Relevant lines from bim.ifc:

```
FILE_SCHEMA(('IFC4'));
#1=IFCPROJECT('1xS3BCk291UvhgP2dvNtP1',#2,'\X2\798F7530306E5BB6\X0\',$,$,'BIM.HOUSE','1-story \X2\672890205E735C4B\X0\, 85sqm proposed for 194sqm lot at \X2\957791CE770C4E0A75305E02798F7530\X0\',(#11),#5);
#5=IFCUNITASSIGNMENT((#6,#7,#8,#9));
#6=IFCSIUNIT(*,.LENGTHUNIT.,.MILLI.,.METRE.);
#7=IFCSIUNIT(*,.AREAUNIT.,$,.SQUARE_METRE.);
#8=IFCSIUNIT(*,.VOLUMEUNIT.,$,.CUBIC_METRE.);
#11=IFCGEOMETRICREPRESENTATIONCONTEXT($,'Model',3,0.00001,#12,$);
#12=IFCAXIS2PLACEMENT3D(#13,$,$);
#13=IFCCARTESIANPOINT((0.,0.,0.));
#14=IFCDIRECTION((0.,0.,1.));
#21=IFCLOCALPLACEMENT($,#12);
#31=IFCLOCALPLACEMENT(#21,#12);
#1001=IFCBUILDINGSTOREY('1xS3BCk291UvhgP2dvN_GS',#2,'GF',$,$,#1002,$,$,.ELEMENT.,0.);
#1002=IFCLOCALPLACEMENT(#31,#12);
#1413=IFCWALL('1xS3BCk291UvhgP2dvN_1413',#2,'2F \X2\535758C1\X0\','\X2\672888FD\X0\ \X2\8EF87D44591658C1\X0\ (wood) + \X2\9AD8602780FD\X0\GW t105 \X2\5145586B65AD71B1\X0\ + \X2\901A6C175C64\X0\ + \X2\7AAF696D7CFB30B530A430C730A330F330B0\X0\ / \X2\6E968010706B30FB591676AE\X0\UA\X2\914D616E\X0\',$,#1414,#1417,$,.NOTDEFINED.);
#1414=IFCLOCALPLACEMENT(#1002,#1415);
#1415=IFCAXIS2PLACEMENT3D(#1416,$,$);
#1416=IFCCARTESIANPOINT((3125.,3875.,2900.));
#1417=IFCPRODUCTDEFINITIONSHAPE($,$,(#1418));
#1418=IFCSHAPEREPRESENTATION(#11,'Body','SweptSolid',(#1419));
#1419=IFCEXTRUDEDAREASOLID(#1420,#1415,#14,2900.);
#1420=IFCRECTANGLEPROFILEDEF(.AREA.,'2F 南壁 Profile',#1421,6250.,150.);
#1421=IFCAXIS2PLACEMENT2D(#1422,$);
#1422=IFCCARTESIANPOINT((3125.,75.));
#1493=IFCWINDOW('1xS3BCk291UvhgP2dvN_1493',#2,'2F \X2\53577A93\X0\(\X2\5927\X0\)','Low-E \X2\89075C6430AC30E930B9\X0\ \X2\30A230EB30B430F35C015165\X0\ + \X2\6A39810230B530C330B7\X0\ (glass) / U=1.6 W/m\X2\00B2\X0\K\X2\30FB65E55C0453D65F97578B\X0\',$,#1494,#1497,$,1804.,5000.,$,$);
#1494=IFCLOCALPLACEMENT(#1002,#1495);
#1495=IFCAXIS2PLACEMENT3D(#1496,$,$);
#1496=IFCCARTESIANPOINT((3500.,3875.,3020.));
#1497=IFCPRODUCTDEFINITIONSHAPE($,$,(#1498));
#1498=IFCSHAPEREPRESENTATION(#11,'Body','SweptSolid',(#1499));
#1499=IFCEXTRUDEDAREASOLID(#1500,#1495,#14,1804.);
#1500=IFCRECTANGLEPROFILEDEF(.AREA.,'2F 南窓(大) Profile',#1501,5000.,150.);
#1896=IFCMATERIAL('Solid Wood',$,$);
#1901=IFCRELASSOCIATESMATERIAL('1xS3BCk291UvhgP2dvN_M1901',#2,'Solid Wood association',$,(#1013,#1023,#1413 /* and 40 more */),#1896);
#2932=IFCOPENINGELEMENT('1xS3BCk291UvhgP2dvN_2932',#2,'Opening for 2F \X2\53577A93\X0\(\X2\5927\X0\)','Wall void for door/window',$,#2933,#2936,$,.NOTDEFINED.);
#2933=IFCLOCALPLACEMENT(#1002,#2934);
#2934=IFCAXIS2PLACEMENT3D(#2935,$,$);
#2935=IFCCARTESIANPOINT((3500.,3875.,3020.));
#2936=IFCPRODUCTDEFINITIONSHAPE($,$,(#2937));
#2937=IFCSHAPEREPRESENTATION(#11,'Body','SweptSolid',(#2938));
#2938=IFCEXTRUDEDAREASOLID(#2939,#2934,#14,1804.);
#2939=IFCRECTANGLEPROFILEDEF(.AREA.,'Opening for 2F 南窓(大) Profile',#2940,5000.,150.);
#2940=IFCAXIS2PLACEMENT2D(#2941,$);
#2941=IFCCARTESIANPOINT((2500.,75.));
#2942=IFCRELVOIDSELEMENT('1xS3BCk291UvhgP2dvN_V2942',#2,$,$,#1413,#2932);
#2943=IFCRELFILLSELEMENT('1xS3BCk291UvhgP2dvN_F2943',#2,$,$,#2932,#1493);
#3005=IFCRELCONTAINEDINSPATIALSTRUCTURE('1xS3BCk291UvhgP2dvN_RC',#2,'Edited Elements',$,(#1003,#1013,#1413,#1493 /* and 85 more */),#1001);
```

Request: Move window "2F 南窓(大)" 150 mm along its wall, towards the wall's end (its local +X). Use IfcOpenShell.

```python
import ifcopenshell
import ifcopenshell.api.geometry
import ifcopenshell.util.placement

model = ifcopenshell.open("bim.ifc")

window = model.by_guid("1xS3BCk291UvhgP2dvN_1493")
opening = window.FillsVoids[0].RelatingOpeningElement
wall = opening.VoidsElements[0].RelatingBuildingElement

wall_matrix = ifcopenshell.util.placement.get_local_placement(wall.ObjectPlacement)
shift = wall_matrix[:3, 0] * 150.0
before = ifcopenshell.util.placement.get_local_placement(window.ObjectPlacement)[:3, 3].copy()

# The window is not placed relative to its opening, so move both.
for product in (opening, window):
    matrix = ifcopenshell.util.placement.get_local_placement(product.ObjectPlacement)
    matrix[:3, 3] += shift
    ifcopenshell.api.geometry.edit_object_placement(model, product=product, matrix=matrix, is_si=False)

after = ifcopenshell.util.placement.get_local_placement(window.ObjectPlacement)[:3, 3]
print("window moved by", (after - before).round(3) + 0.0)

model.write("bim-out.ifc")
```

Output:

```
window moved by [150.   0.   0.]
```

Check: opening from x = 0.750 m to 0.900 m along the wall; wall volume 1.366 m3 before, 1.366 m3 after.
